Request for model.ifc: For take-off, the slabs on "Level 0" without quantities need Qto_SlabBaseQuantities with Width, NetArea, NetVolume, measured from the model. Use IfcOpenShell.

First a look at what the model holds.

```python
import ifcopenshell
import ifcopenshell.util.element
import ifcopenshell.util.unit

model = ifcopenshell.open("model.ifc")
print(model.schema)
for unit_type in ("LENGTHUNIT", "AREAUNIT", "VOLUMEUNIT"):
    print(unit_type, ifcopenshell.util.unit.calculate_unit_scale(model, unit_type))
storey = next(s for s in model.by_type("IfcBuildingStorey") if s.Name == "Level 0")
slabs = [e for e in ifcopenshell.util.element.get_decomposition(storey) if e.is_a("IfcSlab")]
for e in sorted(slabs, key=lambda e: e.id()):
    print(e.id(), e.is_a(), e.Name, list(ifcopenshell.util.element.get_psets(e, qtos_only=True)), sep=" | ")
```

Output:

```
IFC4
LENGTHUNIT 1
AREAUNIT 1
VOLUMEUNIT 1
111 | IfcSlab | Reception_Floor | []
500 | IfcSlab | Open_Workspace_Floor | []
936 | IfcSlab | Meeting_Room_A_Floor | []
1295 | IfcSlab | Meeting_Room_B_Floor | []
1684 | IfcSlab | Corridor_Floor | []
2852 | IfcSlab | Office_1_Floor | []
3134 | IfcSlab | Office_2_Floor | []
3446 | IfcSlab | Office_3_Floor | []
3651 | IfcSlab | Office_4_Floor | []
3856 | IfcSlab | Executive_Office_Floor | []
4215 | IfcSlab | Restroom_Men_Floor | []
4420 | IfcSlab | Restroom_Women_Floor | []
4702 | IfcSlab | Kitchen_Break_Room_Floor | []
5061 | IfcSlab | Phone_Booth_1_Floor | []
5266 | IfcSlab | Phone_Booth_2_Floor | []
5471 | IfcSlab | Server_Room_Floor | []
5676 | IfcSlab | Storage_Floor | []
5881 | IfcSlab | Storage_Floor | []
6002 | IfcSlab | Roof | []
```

```python
import ifcopenshell
import ifcopenshell.api.pset
import ifcopenshell.geom
import ifcopenshell.util.element
import ifcopenshell.util.shape
import ifcopenshell.util.unit

model = ifcopenshell.open("model.ifc")
unit_scale = ifcopenshell.util.unit.calculate_unit_scale(model)
area_scale = ifcopenshell.util.unit.calculate_unit_scale(model, "AREAUNIT")
volume_scale = ifcopenshell.util.unit.calculate_unit_scale(model, "VOLUMEUNIT")
settings = ifcopenshell.geom.settings()

storey = next(s for s in model.by_type("IfcBuildingStorey") if s.Name == "Level 0")
slabs = [e for e in ifcopenshell.util.element.get_decomposition(storey) if e.is_a("IfcSlab")]

for e in sorted(slabs, key=lambda e: e.id()):
    if ifcopenshell.util.element.get_psets(e, qtos_only=True, should_inherit=False):
        continue
    # Geometry comes back in metres, in the element's own axes.
    shape = ifcopenshell.geom.create_shape(settings, e)
    values = {
        "Width": ifcopenshell.util.shape.get_z(shape.geometry) / unit_scale,
        "NetArea": ifcopenshell.util.shape.get_footprint_area(shape.geometry) / area_scale,
        "NetVolume": ifcopenshell.util.shape.get_volume(shape.geometry) / volume_scale,
    }
    qto = ifcopenshell.api.pset.add_qto(model, product=e, name="Qto_SlabBaseQuantities")
    ifcopenshell.api.pset.edit_qto(model, qto=qto, properties=values)
    print(e.id(), {k: round(v, 3) for k, v in values.items()})

model.write("model_rev.ifc")
```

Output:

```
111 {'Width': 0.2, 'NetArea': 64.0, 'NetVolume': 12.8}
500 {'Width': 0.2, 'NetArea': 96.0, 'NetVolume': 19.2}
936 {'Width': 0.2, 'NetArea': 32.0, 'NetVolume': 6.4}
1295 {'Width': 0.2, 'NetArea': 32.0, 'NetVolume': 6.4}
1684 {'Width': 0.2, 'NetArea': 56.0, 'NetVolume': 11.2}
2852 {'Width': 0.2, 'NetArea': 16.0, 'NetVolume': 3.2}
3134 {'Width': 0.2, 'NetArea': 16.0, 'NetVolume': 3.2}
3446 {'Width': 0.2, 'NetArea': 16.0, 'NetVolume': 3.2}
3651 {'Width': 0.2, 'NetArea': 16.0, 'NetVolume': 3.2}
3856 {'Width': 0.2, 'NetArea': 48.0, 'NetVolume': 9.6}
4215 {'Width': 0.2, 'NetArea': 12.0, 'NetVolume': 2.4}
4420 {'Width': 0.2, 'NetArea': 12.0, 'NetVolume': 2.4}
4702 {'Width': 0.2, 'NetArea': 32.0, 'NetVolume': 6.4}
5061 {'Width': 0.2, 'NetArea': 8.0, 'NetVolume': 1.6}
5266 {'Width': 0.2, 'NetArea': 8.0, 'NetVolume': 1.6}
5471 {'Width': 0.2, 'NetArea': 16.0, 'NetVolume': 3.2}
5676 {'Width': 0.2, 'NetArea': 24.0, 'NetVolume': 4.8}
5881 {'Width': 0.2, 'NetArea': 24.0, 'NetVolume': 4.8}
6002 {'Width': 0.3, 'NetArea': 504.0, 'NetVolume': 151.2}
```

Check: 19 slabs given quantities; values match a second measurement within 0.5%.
